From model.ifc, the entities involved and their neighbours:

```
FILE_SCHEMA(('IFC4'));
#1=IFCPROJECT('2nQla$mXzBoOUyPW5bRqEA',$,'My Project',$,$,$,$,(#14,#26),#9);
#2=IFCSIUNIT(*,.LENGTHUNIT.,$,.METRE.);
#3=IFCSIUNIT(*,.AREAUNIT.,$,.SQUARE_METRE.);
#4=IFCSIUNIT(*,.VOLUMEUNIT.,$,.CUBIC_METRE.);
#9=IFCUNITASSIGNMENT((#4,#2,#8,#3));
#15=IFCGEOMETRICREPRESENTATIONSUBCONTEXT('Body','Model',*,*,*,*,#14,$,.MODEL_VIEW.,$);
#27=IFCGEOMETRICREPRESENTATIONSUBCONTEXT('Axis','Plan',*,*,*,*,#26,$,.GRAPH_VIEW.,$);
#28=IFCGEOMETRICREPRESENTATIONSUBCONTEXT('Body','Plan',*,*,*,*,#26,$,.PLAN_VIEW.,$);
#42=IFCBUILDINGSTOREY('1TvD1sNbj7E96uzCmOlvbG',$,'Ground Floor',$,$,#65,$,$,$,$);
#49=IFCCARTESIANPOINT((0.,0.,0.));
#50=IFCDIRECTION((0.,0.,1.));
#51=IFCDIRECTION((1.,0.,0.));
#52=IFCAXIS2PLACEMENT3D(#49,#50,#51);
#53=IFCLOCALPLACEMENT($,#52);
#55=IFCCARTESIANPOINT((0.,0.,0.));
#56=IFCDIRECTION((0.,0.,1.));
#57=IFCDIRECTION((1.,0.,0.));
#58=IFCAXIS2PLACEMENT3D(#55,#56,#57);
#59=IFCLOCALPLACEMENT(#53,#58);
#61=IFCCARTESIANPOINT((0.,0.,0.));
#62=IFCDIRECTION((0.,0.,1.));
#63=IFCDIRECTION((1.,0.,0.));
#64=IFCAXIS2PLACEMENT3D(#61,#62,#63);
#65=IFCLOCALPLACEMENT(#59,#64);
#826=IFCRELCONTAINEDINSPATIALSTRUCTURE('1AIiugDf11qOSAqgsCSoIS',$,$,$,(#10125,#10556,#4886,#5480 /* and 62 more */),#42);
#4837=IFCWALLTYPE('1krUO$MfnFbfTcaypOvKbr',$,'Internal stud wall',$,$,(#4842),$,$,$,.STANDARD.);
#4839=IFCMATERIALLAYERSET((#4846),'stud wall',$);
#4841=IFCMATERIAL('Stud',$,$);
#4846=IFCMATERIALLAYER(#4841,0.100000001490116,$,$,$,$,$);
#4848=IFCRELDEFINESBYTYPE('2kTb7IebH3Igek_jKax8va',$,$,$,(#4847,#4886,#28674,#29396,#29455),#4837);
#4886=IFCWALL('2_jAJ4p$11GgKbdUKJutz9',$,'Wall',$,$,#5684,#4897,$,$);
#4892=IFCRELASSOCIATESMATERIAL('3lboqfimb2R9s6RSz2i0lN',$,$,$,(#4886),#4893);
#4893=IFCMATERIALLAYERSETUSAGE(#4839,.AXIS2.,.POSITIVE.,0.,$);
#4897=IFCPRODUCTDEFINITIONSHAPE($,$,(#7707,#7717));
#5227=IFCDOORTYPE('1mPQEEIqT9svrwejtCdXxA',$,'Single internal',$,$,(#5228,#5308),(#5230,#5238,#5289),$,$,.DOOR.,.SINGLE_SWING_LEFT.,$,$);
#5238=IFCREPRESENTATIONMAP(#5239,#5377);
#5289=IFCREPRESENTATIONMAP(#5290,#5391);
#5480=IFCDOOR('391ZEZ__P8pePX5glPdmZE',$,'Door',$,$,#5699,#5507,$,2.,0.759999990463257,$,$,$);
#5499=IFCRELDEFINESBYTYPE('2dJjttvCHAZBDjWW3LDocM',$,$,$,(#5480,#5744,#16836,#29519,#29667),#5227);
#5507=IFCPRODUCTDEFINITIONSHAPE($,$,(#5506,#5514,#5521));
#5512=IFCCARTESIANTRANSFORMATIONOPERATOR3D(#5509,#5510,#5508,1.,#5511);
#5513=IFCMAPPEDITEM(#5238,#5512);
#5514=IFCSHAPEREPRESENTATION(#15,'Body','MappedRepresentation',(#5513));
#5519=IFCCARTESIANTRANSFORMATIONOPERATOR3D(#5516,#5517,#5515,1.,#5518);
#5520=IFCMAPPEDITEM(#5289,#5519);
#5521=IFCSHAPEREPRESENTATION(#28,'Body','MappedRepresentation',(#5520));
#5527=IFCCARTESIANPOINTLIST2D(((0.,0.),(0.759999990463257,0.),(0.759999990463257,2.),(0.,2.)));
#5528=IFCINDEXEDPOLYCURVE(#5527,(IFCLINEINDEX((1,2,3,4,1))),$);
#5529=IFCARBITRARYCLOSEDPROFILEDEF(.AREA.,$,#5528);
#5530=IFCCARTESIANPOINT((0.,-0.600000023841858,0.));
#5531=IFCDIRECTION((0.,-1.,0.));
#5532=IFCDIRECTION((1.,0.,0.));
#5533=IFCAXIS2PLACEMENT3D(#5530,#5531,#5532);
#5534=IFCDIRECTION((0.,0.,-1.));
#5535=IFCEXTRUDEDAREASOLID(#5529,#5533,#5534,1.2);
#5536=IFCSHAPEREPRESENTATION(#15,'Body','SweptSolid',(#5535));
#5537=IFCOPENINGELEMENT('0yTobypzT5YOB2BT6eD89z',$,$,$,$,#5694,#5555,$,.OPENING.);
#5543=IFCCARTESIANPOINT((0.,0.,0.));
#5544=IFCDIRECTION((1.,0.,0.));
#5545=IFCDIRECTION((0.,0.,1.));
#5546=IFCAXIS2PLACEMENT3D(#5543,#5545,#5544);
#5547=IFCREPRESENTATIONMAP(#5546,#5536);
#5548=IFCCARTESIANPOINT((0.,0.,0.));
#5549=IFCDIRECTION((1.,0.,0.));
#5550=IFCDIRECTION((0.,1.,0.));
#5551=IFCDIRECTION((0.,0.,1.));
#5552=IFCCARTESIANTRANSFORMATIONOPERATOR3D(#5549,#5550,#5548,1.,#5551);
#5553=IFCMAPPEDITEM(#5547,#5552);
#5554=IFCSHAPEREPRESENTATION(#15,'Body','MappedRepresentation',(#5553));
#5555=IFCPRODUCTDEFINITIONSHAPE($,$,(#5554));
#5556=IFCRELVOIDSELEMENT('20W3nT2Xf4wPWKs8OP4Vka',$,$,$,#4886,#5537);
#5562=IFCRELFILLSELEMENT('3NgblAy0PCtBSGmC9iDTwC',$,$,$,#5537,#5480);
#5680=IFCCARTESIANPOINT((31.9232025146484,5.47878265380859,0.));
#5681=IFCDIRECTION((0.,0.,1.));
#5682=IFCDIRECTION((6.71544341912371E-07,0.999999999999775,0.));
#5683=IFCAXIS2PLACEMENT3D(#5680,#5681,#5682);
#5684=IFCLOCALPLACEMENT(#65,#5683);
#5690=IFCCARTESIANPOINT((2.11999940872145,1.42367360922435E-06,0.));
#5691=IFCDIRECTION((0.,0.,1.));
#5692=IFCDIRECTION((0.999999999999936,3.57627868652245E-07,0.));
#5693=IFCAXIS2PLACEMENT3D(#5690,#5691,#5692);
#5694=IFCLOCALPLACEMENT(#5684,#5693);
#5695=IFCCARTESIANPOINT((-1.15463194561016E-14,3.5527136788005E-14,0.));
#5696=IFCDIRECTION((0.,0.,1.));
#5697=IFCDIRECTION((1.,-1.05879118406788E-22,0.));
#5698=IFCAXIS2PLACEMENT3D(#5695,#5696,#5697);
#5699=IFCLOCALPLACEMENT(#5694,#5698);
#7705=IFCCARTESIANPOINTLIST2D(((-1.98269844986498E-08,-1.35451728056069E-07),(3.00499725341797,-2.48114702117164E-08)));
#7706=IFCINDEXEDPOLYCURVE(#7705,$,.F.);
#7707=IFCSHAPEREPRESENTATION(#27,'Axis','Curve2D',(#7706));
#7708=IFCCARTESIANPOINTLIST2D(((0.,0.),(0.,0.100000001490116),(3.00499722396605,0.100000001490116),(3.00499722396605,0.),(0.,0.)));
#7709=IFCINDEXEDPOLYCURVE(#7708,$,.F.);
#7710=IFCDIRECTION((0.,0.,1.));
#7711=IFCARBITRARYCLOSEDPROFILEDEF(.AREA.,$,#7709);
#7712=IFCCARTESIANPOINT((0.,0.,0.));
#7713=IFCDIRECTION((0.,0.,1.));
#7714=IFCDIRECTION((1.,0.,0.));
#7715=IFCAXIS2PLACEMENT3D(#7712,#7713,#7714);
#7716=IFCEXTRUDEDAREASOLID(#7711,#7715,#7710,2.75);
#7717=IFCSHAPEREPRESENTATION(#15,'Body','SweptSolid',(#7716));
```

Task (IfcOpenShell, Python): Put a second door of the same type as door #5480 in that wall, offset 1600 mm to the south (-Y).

```python
import ifcopenshell
import ifcopenshell.api.feature
import ifcopenshell.api.geometry
import ifcopenshell.api.root
import ifcopenshell.geom
import ifcopenshell.util.element
import ifcopenshell.util.placement
import ifcopenshell.util.shape

model = ifcopenshell.open("model.ifc")
settings = ifcopenshell.geom.settings()


def volume(element):
    """Net volume in cubic metres, openings subtracted."""
    shape = ifcopenshell.geom.create_shape(settings, element)
    return ifcopenshell.util.shape.get_volume(shape.geometry)


door = model.by_guid("391ZEZ__P8pePX5glPdmZE")
opening = door.FillsVoids[0].RelatingOpeningElement
wall = opening.VoidsElements[0].RelatingBuildingElement
before = volume(wall)
shift = ifcopenshell.util.placement.get_local_placement(wall.ObjectPlacement)[:3, 0] * -1.6

# copy_class copies the void relationship, type, container and properties, but no geometry.
new_opening = ifcopenshell.api.root.copy_class(model, product=opening)
new_opening.Representation = ifcopenshell.util.element.copy_deep(
    model, opening.Representation, exclude=["IfcGeometricRepresentationContext", "IfcRepresentationMap"]
)
new_door = ifcopenshell.api.root.copy_class(model, product=door)
new_door.Representation = ifcopenshell.util.element.copy_deep(
    model, door.Representation, exclude=["IfcGeometricRepresentationContext", "IfcRepresentationMap"]
)
ifcopenshell.api.feature.add_filling(model, opening=new_opening, element=new_door)

for old, new in ((opening, new_opening), (door, new_door)):
    matrix = ifcopenshell.util.placement.get_local_placement(old.ObjectPlacement)
    matrix[:3, 3] += shift
    ifcopenshell.api.geometry.edit_object_placement(model, product=new, matrix=matrix, is_si=False)

after = volume(wall)

print(f"wall volume {before:.3f} -> {after:.3f} m3")

model.write("model_v2.ifc")
```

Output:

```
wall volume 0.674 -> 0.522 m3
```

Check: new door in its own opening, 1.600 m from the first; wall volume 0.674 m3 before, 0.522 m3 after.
